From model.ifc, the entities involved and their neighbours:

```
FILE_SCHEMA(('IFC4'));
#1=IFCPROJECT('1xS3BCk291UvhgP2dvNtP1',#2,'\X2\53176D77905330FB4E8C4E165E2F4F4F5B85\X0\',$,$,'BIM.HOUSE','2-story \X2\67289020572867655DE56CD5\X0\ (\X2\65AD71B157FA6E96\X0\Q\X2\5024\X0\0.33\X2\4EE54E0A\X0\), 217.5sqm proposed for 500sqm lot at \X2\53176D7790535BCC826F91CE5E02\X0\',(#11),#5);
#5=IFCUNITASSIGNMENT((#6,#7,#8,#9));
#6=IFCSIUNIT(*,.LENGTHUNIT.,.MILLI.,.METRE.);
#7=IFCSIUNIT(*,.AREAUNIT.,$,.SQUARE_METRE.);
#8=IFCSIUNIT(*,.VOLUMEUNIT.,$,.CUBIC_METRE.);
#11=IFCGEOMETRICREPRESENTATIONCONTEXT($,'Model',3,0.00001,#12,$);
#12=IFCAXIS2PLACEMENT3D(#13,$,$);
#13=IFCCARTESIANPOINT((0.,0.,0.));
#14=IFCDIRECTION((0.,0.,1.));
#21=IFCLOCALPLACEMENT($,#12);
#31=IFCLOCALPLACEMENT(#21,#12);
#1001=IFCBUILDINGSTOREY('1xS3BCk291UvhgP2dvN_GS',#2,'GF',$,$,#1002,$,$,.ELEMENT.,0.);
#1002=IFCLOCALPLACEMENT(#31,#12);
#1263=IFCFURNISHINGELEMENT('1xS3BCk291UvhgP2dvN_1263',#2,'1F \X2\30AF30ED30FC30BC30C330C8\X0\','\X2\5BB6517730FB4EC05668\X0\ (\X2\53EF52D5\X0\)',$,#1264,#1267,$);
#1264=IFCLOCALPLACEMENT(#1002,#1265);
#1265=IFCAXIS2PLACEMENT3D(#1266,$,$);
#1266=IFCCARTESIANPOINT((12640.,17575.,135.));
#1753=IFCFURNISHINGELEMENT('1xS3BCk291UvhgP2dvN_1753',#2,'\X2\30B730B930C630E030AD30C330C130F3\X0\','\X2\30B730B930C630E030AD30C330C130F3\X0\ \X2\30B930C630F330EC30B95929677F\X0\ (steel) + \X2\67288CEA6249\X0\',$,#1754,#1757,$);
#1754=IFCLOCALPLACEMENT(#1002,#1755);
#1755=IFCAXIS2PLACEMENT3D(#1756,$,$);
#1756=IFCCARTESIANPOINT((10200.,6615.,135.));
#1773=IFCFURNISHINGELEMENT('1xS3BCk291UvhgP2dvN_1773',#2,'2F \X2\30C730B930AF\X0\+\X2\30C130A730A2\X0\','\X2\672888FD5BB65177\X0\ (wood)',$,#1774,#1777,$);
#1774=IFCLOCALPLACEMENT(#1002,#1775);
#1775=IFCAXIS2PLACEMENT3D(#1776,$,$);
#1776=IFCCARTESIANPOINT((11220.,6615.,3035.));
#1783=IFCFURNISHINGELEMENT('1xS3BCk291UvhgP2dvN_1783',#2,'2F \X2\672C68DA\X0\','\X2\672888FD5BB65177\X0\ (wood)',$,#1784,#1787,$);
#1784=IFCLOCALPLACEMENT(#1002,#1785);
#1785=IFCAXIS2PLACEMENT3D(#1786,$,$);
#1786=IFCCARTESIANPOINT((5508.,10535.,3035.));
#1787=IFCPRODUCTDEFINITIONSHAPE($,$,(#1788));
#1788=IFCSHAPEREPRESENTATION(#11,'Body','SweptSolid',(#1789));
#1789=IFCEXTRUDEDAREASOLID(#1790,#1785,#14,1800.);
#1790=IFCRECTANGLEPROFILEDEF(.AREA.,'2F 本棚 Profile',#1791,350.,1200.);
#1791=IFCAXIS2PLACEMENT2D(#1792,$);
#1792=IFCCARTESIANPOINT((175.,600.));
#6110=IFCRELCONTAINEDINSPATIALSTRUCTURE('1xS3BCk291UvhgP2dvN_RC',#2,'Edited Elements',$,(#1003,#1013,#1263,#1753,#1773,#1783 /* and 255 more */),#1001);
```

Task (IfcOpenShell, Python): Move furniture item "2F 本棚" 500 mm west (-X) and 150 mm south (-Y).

```python
import ifcopenshell
import ifcopenshell.api.geometry
import ifcopenshell.util.placement

model = ifcopenshell.open("model.ifc")

item = model.by_id(1783)
matrix = ifcopenshell.util.placement.get_local_placement(item.ObjectPlacement)
matrix[0, 3] -= 500.0
matrix[1, 3] -= 150.0
ifcopenshell.api.geometry.edit_object_placement(model, product=item, matrix=matrix, is_si=False)

print(ifcopenshell.util.placement.get_local_placement(item.ObjectPlacement).round(3) + 0.0)

model.write("model_updated.ifc")
```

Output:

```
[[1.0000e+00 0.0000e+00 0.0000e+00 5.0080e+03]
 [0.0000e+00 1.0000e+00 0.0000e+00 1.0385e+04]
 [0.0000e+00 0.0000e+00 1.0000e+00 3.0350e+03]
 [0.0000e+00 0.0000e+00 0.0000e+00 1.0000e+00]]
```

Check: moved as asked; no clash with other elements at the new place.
